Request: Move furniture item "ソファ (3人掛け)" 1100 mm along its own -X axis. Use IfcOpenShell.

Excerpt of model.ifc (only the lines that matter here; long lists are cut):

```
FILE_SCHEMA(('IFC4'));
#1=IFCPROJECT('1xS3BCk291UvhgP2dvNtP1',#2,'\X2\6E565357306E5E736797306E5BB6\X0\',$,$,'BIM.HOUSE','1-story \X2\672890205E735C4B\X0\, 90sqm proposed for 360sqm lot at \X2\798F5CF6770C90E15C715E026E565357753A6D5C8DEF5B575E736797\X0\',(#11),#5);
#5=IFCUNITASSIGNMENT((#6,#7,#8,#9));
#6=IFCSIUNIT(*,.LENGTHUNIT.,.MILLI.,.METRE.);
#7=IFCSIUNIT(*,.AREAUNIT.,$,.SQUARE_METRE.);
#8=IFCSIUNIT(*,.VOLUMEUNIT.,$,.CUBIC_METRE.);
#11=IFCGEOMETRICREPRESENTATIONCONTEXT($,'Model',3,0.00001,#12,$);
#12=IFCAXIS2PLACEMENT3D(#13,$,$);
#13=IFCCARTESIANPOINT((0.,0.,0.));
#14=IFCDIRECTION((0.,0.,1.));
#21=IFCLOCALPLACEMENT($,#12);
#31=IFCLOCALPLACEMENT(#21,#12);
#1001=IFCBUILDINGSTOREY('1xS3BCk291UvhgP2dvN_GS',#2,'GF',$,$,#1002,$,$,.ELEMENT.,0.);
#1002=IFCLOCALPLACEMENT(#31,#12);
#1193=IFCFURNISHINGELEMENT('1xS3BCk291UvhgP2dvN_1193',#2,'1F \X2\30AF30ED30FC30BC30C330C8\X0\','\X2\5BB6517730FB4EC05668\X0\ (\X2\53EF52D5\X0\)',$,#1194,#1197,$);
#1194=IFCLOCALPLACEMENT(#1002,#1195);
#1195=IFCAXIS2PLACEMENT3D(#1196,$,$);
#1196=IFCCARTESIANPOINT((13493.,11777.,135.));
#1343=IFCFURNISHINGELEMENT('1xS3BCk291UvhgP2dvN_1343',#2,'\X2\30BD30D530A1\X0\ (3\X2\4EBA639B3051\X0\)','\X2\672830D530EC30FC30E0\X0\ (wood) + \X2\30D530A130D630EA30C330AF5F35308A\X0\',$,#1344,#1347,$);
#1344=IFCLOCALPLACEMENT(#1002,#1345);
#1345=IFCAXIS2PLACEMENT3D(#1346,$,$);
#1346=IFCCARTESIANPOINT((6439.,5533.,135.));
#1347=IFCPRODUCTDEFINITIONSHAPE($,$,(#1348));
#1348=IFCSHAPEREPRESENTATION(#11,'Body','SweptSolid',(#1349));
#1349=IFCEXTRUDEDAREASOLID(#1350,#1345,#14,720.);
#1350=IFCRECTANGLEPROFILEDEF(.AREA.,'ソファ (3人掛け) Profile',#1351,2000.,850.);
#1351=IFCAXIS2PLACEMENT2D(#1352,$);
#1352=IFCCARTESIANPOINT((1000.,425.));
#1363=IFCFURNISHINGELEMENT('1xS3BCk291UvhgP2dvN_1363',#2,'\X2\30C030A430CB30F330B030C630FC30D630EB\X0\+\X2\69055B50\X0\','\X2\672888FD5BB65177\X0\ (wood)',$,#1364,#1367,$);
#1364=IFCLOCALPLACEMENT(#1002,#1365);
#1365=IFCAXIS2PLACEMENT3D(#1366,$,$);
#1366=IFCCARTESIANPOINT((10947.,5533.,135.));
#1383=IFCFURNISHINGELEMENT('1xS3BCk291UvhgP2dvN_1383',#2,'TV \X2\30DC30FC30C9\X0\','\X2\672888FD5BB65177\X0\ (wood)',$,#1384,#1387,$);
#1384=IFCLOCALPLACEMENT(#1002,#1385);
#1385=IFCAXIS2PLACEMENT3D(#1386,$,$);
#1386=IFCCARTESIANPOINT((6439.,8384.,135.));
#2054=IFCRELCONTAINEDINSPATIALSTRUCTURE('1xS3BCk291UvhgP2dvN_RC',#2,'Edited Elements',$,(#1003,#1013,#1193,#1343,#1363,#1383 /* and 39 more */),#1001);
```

```python
import ifcopenshell
import ifcopenshell.api.geometry
import ifcopenshell.util.placement
import ifcopenshell.util.unit

model = ifcopenshell.open("model.ifc")
unit_scale = ifcopenshell.util.unit.calculate_unit_scale(model)

item = model.by_guid("1xS3BCk291UvhgP2dvN_1343")
matrix = ifcopenshell.util.placement.get_local_placement(item.ObjectPlacement)
matrix[:3, 3] -= matrix[:3, 0] * 1.1 / unit_scale
ifcopenshell.api.geometry.edit_object_placement(model, product=item, matrix=matrix, is_si=False)

print(ifcopenshell.util.placement.get_local_placement(item.ObjectPlacement).round(3) + 0.0)

model.write("model_rev.ifc")
```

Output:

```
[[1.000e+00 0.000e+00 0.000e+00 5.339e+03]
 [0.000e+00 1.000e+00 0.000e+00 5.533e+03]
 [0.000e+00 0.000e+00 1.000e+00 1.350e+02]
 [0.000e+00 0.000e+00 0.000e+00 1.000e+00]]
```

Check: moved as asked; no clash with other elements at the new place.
